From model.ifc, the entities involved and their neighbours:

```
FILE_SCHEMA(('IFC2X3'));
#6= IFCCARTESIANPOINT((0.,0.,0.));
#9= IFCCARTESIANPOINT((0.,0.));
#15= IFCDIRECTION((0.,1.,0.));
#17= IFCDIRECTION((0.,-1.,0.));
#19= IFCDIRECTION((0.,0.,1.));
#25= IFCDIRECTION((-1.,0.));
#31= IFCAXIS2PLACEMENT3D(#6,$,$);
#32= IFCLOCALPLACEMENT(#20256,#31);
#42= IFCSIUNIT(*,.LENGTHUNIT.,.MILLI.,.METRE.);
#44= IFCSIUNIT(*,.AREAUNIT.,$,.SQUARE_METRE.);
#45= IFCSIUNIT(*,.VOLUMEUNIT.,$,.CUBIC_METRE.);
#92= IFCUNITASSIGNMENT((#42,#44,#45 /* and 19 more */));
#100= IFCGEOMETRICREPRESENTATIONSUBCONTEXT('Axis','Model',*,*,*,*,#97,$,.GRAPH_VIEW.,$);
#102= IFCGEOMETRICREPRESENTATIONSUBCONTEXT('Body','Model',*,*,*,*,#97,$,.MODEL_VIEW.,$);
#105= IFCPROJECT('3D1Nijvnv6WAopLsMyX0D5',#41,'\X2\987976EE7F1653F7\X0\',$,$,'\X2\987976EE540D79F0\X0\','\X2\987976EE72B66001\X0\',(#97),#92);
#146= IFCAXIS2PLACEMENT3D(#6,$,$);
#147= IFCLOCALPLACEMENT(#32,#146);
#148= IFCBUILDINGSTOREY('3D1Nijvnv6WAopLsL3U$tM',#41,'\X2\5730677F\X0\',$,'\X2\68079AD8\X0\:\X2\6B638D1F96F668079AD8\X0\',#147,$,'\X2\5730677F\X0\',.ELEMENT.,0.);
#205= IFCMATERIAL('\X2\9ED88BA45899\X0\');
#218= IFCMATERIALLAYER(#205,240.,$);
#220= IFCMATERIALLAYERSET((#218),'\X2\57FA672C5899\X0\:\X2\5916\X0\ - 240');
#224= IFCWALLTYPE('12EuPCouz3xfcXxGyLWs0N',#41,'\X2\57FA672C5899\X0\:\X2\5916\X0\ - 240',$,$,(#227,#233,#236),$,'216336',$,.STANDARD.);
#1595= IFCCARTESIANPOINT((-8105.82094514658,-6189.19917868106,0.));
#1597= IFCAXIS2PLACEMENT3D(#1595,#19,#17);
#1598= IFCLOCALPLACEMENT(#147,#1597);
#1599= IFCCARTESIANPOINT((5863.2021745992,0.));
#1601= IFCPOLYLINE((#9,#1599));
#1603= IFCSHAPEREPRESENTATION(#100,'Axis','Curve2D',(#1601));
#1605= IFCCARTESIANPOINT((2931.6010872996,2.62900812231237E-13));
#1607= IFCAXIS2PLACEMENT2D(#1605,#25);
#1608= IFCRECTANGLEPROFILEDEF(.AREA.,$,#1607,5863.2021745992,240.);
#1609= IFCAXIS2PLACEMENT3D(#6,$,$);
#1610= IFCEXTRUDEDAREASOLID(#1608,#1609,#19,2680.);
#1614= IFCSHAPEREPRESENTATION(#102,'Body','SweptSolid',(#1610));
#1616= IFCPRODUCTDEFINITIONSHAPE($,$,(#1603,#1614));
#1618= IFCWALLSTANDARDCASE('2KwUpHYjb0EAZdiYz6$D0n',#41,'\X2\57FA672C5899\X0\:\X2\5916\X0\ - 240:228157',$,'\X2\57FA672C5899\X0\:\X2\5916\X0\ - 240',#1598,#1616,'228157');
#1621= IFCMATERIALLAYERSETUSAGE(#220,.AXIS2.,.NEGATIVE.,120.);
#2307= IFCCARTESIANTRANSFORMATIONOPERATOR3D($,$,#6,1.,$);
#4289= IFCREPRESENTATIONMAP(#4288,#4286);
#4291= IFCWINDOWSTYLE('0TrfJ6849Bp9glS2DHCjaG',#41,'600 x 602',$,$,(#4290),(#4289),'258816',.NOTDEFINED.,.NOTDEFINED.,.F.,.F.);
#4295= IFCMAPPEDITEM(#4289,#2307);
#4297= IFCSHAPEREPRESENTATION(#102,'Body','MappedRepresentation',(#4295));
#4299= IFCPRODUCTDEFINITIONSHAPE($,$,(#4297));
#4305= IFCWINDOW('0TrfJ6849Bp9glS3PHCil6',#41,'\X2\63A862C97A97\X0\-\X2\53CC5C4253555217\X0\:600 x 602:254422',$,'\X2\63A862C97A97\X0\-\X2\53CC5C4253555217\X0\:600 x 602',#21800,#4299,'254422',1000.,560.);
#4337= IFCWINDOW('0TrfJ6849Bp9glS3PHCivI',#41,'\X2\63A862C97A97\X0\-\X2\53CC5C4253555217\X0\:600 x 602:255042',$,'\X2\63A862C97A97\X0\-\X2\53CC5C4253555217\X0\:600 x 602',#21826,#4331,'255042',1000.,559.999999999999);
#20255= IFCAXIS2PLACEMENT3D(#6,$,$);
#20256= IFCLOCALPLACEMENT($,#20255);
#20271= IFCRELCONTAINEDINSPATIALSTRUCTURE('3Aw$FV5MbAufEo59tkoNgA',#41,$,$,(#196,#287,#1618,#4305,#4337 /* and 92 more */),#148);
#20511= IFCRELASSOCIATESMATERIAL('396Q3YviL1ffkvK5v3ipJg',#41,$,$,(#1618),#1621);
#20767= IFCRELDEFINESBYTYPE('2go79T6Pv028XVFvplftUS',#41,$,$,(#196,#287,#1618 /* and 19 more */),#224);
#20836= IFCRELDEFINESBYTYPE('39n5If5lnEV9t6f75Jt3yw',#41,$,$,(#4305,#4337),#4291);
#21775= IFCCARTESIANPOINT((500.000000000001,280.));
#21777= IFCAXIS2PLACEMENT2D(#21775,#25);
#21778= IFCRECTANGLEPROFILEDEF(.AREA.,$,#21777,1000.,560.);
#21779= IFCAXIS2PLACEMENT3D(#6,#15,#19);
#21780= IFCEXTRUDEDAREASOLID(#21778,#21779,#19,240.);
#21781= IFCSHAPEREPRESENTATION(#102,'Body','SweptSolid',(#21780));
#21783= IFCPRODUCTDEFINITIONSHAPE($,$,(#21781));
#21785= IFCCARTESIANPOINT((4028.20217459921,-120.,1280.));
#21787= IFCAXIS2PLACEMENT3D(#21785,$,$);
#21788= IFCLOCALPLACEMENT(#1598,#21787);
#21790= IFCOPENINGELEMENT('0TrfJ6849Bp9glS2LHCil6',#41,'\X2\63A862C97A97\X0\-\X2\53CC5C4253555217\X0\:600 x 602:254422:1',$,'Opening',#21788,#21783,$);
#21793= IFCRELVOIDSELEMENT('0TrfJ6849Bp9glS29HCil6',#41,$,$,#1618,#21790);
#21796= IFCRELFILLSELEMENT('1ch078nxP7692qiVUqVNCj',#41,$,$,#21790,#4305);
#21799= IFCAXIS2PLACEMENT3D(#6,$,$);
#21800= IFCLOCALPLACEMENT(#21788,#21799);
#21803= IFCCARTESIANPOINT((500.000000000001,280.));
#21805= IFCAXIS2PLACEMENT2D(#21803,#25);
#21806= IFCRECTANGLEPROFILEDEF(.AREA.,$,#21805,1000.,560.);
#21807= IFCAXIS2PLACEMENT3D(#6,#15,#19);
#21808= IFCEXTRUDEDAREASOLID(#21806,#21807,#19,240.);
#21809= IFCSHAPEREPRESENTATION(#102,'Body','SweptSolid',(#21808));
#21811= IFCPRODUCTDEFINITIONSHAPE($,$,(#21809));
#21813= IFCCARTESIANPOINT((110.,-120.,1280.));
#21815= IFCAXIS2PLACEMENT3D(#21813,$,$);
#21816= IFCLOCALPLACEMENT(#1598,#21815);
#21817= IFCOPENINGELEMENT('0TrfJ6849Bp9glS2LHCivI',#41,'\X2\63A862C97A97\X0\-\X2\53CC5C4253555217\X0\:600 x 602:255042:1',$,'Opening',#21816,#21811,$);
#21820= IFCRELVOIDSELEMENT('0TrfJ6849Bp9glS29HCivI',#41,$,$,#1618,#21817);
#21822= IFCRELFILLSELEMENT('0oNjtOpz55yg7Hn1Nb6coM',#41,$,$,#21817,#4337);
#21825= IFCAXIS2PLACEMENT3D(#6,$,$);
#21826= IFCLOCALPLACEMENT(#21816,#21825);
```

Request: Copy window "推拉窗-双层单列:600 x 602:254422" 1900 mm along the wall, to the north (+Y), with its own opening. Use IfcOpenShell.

```python
import ifcopenshell
import ifcopenshell.api.feature
import ifcopenshell.api.geometry
import ifcopenshell.api.root
import ifcopenshell.geom
import ifcopenshell.util.element
import ifcopenshell.util.placement
import ifcopenshell.util.shape
import ifcopenshell.util.unit

model = ifcopenshell.open("model.ifc")
unit_scale = ifcopenshell.util.unit.calculate_unit_scale(model)
settings = ifcopenshell.geom.settings()


def volume(element):
    """Net volume in cubic metres, openings subtracted."""
    shape = ifcopenshell.geom.create_shape(settings, element)
    return ifcopenshell.util.shape.get_volume(shape.geometry)


def reuse_history(source, copy):
    """copy_class also copies each property set's owner history, people and application; keep the originals."""
    for rel in copy.IsDefinedBy:
        if rel.is_a("IfcRelDefinesByProperties") and (history := rel.RelatingPropertyDefinition.OwnerHistory):
            rel.RelatingPropertyDefinition.OwnerHistory = source.OwnerHistory
            ifcopenshell.util.element.remove_deep2(model, history)


window = model.by_guid("0TrfJ6849Bp9glS3PHCil6")
opening = window.FillsVoids[0].RelatingOpeningElement
wall = opening.VoidsElements[0].RelatingBuildingElement
before = volume(wall)
shift = ifcopenshell.util.placement.get_local_placement(wall.ObjectPlacement)[:3, 0] * -1.9 / unit_scale

# copy_class copies the void relationship, type, container and properties, but no geometry.
new_opening = ifcopenshell.api.root.copy_class(model, product=opening)
new_opening.Representation = ifcopenshell.util.element.copy_deep(
    model, opening.Representation, exclude=["IfcGeometricRepresentationContext", "IfcRepresentationMap"]
)
new_opening.Name = "推拉窗-双层单列:600 x 602"
new_window = ifcopenshell.api.root.copy_class(model, product=window)
new_window.Representation = ifcopenshell.util.element.copy_deep(
    model, window.Representation, exclude=["IfcGeometricRepresentationContext", "IfcRepresentationMap"]
)
new_window.Name = "推拉窗-双层单列:600 x 602"
new_window.Tag = None
reuse_history(window, new_window)
fills = ifcopenshell.api.feature.add_filling(model, opening=new_opening, element=new_window)
fills.OwnerHistory = new_window.OwnerHistory  # required in IFC2X3

for old, new in ((opening, new_opening), (window, new_window)):
    matrix = ifcopenshell.util.placement.get_local_placement(old.ObjectPlacement)
    matrix[:3, 3] += shift
    ifcopenshell.api.geometry.edit_object_placement(model, product=new, matrix=matrix, is_si=False)

after = volume(wall)

print(f"wall volume {before:.3f} -> {after:.3f} m3")

model.write("model_rev.ifc")
```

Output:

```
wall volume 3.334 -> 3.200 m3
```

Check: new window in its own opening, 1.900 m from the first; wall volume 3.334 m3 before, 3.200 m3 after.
